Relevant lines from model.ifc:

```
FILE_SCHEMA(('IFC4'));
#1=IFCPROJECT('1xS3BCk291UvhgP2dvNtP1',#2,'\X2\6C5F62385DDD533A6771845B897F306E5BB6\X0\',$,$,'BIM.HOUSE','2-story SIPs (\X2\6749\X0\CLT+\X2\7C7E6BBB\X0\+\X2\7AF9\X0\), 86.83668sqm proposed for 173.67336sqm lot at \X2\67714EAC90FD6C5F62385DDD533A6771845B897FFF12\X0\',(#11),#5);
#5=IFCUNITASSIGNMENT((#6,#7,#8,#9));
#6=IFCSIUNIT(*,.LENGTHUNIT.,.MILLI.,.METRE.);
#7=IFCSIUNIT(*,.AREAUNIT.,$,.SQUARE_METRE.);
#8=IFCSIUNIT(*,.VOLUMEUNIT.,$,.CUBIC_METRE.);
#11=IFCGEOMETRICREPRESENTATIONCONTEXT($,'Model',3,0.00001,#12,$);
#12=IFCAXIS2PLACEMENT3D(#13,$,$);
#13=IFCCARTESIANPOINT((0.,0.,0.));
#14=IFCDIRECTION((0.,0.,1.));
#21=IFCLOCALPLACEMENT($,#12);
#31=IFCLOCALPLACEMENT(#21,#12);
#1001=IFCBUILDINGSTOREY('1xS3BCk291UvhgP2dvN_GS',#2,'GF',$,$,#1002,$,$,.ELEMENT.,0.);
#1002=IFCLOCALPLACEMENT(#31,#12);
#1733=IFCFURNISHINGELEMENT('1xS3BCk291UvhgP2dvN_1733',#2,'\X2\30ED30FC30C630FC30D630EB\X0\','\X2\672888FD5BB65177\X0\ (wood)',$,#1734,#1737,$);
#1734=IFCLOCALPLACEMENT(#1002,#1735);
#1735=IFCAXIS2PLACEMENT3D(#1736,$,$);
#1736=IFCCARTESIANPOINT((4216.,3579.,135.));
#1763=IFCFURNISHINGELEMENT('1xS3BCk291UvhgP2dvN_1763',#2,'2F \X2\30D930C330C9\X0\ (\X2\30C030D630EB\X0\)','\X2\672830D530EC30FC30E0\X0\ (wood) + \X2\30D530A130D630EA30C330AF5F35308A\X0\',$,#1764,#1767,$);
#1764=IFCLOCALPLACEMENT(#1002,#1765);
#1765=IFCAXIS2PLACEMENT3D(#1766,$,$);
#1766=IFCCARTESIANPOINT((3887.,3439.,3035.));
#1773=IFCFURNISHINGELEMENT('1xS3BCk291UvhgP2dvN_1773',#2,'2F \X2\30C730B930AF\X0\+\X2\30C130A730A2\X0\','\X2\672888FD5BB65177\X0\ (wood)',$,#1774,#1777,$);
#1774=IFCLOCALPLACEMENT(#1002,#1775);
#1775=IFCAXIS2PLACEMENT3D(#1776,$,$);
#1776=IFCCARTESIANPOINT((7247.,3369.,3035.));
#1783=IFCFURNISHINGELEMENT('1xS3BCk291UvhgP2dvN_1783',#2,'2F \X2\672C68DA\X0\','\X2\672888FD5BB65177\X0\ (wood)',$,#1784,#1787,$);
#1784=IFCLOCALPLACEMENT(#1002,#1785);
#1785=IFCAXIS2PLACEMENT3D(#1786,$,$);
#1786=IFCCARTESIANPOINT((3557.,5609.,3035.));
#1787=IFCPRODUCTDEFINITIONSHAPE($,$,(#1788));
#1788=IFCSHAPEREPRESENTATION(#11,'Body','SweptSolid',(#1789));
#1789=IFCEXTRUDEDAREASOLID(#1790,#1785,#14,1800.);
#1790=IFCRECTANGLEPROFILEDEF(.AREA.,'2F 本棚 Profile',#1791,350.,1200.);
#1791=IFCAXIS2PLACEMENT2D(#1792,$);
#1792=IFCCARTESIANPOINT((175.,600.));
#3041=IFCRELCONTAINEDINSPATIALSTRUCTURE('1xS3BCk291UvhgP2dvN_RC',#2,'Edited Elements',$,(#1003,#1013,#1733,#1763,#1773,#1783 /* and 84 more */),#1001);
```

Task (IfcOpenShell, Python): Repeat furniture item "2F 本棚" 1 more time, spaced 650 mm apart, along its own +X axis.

```python
import ifcopenshell
import ifcopenshell.api.geometry
import ifcopenshell.api.root
import ifcopenshell.util.element
import ifcopenshell.util.placement
import ifcopenshell.util.unit

model = ifcopenshell.open("model.ifc")
unit_scale = ifcopenshell.util.unit.calculate_unit_scale(model)


def reuse_history(source, copy):
    """copy_class also copies each property set's owner history, people and application; keep the originals."""
    for rel in copy.IsDefinedBy:
        if rel.is_a("IfcRelDefinesByProperties") and (history := rel.RelatingPropertyDefinition.OwnerHistory):
            rel.RelatingPropertyDefinition.OwnerHistory = source.OwnerHistory
            ifcopenshell.util.element.remove_deep2(model, history)


source = model.by_guid("1xS3BCk291UvhgP2dvN_1783")
base = ifcopenshell.util.placement.get_local_placement(source.ObjectPlacement)
step = base[:3, 0] * 0.65 / unit_scale

for i in range(1, 2):
    copy = ifcopenshell.api.root.copy_class(model, product=source)
    copy.Representation = ifcopenshell.util.element.copy_deep(
        model, source.Representation, exclude=["IfcGeometricRepresentationContext", "IfcRepresentationMap"]
    )
    reuse_history(source, copy)
    matrix = base.copy()
    matrix[:3, 3] += i * step
    print("added at", matrix[:3, 3].round(3) + 0.0)
    ifcopenshell.api.geometry.edit_object_placement(model, product=copy, matrix=matrix, is_si=False)

model.write("model_edited.ifc")
```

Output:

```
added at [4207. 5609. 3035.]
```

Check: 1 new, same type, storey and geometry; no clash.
